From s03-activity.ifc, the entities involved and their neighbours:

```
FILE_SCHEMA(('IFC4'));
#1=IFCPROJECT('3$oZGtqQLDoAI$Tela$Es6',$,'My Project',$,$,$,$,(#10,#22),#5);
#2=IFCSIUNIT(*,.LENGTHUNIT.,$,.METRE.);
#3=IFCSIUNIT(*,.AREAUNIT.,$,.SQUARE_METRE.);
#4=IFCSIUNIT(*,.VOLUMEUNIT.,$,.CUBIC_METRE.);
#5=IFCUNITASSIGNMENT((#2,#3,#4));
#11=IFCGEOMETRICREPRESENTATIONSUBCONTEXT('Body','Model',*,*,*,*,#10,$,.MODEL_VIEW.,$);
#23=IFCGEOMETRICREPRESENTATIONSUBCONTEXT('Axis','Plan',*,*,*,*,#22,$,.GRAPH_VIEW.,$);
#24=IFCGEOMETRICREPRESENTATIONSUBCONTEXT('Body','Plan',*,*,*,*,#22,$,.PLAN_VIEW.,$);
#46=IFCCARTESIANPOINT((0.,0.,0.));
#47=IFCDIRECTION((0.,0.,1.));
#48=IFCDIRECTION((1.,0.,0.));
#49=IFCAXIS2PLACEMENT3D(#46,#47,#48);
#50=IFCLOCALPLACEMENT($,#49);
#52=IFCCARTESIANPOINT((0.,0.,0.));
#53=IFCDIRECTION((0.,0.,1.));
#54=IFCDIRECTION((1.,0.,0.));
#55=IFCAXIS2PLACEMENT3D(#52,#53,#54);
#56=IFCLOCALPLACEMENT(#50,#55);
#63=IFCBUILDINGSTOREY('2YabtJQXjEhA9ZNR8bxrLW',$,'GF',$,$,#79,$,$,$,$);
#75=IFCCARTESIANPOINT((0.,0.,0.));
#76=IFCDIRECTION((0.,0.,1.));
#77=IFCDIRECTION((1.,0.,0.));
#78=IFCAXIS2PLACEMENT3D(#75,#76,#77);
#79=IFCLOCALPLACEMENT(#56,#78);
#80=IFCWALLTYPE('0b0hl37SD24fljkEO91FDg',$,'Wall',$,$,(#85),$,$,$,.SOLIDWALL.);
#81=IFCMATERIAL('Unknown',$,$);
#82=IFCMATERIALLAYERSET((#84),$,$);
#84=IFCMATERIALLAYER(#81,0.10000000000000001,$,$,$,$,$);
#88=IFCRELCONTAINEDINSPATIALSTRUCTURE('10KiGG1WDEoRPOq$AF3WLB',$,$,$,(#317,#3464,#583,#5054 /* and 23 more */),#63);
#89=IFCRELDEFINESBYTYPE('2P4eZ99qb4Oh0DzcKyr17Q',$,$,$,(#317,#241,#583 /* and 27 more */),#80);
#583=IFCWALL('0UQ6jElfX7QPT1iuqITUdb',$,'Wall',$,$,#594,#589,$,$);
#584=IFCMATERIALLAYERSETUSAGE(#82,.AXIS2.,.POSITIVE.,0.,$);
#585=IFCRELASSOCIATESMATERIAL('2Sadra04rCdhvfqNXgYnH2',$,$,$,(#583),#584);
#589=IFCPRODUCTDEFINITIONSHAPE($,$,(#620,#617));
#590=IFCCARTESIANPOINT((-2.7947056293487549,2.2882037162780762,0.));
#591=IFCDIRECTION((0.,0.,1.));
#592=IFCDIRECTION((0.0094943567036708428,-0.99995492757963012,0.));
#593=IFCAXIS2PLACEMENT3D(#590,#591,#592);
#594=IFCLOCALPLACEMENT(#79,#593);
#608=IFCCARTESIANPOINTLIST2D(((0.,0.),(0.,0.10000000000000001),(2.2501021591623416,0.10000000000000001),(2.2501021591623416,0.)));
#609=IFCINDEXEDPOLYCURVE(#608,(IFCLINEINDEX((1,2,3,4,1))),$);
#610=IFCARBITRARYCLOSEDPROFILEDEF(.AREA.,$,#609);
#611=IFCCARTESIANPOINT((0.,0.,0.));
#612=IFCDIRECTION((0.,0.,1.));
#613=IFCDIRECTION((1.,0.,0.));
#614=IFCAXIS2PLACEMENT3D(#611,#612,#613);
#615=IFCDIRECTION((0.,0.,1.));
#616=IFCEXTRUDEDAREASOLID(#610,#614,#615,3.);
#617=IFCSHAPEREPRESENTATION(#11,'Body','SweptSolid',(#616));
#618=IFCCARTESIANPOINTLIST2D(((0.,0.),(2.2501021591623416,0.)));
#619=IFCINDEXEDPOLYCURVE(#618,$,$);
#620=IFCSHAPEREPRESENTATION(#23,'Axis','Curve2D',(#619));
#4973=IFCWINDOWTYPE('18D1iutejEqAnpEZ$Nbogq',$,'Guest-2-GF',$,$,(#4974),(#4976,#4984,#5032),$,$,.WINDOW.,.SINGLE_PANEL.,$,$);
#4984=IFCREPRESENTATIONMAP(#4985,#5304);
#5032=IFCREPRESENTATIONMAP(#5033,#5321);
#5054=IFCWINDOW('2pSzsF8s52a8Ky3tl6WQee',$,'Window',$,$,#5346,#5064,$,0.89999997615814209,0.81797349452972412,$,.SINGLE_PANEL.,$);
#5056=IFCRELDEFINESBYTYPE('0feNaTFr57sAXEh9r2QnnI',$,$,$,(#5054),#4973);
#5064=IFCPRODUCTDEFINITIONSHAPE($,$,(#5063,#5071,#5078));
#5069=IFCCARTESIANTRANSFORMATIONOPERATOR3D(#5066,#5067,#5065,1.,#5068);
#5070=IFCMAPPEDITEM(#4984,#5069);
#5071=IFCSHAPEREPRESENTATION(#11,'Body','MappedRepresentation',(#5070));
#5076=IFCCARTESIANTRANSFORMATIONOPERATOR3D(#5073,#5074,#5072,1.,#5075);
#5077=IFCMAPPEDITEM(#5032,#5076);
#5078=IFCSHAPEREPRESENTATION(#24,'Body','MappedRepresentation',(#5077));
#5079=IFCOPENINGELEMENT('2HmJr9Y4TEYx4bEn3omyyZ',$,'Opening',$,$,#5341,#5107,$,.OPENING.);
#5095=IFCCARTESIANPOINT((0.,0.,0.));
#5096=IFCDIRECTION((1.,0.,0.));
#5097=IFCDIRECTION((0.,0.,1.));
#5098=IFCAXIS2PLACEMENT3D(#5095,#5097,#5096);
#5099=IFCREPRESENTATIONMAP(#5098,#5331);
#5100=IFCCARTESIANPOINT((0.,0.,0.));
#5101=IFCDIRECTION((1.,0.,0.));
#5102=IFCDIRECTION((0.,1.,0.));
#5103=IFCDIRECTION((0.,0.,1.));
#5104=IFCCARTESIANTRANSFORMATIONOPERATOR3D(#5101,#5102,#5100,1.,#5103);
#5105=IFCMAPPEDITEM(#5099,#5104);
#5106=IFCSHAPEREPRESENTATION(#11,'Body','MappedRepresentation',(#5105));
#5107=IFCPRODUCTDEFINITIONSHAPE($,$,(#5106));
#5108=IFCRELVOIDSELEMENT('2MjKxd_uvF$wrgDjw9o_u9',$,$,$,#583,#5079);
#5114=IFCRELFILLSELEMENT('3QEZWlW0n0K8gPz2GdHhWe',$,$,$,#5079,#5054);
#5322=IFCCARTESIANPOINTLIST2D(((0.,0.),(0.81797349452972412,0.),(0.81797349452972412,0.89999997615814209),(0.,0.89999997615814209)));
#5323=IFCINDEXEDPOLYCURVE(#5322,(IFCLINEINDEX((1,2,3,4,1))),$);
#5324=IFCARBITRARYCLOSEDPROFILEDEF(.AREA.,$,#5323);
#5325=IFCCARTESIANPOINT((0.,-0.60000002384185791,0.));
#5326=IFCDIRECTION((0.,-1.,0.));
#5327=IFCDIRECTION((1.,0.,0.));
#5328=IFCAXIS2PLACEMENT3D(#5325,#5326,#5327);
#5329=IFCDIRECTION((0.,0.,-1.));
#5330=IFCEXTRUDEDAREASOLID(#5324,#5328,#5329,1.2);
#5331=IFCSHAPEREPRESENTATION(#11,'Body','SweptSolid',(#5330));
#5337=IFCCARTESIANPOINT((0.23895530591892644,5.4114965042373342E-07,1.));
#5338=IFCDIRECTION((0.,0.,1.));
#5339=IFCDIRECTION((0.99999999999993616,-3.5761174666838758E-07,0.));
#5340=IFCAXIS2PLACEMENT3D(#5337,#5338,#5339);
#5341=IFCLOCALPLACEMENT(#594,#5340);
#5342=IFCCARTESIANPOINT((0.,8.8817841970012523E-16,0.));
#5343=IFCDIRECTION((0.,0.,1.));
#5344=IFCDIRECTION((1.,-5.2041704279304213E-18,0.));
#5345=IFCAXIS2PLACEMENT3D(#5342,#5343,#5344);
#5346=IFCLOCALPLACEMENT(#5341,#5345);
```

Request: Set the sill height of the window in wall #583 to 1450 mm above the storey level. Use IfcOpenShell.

```python
import numpy as np
import ifcopenshell
import ifcopenshell.api.geometry
import ifcopenshell.geom
import ifcopenshell.util.element
import ifcopenshell.util.placement
import ifcopenshell.util.shape
import ifcopenshell.util.unit

model = ifcopenshell.open("s03-activity.ifc")
unit_scale = ifcopenshell.util.unit.calculate_unit_scale(model)

window = model.by_guid("2pSzsF8s52a8Ky3tl6WQee")
opening = window.FillsVoids[0].RelatingOpeningElement
storey = ifcopenshell.util.element.get_container(window, ifc_class="IfcBuildingStorey")
level = ifcopenshell.util.placement.get_local_placement(storey.ObjectPlacement)[2, 3]

# The opening's origin need not be at the sill, so measure its lowest point.
shape = ifcopenshell.geom.create_shape(ifcopenshell.geom.settings(), opening)
bottom = ifcopenshell.util.shape.get_shape_bottom_elevation(shape, shape.geometry) / unit_scale
dz = level + 1.45 - bottom

shift = np.array([0.0, 0.0, dz])
# The window is placed relative to its opening, so it follows when the opening moves.
matrix = ifcopenshell.util.placement.get_local_placement(opening.ObjectPlacement)
matrix[:3, 3] += shift
ifcopenshell.api.geometry.edit_object_placement(
    model, product=opening, matrix=matrix, is_si=False, should_transform_children=True
)

print(f"moved by {dz * unit_scale:+.3f} m")

model.write("s03-activity_edited.ifc")
```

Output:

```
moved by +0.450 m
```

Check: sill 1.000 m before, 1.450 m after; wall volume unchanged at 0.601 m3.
